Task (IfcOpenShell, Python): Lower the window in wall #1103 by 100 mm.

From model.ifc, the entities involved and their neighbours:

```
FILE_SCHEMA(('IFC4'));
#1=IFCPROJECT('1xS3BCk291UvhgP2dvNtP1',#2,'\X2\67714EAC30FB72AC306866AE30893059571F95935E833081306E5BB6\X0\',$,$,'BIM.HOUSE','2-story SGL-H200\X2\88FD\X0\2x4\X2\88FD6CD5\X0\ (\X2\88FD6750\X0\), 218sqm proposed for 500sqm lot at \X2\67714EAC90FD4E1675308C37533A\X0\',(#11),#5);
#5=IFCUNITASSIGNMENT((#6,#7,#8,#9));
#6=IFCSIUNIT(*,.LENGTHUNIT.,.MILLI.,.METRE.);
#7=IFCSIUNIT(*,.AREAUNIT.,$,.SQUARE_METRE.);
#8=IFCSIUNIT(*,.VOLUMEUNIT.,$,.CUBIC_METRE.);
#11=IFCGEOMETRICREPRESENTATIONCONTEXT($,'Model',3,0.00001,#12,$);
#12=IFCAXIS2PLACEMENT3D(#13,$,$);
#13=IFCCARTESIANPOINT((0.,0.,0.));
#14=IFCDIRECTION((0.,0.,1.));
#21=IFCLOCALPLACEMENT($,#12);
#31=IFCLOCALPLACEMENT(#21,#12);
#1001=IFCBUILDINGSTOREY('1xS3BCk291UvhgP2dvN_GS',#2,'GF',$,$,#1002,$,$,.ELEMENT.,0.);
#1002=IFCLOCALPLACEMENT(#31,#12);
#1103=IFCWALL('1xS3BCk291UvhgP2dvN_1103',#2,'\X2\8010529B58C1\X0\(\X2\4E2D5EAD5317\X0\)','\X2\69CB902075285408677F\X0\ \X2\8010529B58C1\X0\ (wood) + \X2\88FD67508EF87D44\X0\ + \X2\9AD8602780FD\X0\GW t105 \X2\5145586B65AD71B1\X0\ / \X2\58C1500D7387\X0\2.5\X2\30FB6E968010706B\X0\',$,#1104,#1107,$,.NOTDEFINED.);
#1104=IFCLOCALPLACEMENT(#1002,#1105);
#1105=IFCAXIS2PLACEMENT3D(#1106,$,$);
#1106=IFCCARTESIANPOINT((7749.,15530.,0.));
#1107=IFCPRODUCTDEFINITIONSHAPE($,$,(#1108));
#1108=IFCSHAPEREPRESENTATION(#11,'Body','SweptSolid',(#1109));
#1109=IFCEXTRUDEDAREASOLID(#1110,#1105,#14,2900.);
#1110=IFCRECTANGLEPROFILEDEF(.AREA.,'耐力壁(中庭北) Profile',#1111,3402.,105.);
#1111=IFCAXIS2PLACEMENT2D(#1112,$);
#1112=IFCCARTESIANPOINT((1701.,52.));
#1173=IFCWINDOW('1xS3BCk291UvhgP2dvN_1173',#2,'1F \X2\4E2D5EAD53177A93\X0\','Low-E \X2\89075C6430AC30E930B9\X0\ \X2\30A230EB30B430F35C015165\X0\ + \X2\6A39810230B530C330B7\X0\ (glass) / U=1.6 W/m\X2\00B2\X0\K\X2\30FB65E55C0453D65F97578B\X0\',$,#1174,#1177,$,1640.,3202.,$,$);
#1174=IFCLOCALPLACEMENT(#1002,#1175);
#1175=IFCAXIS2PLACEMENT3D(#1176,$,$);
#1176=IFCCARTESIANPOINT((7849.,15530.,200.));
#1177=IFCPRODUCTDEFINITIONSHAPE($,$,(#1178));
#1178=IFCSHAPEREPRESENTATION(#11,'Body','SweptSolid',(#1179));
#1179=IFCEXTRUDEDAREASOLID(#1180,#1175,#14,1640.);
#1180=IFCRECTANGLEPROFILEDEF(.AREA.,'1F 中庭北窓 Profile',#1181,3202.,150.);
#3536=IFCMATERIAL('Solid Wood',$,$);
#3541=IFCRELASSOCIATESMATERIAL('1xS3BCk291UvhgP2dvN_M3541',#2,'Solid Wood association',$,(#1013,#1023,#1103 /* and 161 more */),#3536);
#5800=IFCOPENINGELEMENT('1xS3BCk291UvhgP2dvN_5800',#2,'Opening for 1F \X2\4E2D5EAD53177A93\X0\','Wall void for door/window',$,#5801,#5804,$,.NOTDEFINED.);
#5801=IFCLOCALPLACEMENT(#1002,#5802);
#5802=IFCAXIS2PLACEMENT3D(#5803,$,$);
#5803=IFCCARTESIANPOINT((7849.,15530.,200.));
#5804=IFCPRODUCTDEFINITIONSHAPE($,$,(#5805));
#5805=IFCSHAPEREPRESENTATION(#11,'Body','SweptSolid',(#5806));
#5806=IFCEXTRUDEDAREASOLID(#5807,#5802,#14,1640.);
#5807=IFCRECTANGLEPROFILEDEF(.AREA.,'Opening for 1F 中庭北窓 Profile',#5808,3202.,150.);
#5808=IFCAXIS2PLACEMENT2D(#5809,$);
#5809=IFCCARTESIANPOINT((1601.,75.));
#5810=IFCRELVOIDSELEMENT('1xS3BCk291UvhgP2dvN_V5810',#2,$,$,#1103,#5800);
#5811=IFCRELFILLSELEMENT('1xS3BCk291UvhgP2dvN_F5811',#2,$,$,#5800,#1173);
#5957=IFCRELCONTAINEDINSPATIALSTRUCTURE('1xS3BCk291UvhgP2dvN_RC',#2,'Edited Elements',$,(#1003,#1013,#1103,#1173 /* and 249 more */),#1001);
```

```python
import numpy as np
import ifcopenshell
import ifcopenshell.api.geometry
import ifcopenshell.util.placement
import ifcopenshell.util.unit

model = ifcopenshell.open("model.ifc")
unit_scale = ifcopenshell.util.unit.calculate_unit_scale(model)

window = model.by_guid("1xS3BCk291UvhgP2dvN_1173")
opening = window.FillsVoids[0].RelatingOpeningElement
dz = -100.0

shift = np.array([0.0, 0.0, dz])
# The window is not placed relative to its opening, so move both.
for product in (opening, window):
    matrix = ifcopenshell.util.placement.get_local_placement(product.ObjectPlacement)
    matrix[:3, 3] += shift
    ifcopenshell.api.geometry.edit_object_placement(model, product=product, matrix=matrix, is_si=False)

print(f"moved by {dz * unit_scale:+.3f} m")

model.write("model_v2.ifc")
```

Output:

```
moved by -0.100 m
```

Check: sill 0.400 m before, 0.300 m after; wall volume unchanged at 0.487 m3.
